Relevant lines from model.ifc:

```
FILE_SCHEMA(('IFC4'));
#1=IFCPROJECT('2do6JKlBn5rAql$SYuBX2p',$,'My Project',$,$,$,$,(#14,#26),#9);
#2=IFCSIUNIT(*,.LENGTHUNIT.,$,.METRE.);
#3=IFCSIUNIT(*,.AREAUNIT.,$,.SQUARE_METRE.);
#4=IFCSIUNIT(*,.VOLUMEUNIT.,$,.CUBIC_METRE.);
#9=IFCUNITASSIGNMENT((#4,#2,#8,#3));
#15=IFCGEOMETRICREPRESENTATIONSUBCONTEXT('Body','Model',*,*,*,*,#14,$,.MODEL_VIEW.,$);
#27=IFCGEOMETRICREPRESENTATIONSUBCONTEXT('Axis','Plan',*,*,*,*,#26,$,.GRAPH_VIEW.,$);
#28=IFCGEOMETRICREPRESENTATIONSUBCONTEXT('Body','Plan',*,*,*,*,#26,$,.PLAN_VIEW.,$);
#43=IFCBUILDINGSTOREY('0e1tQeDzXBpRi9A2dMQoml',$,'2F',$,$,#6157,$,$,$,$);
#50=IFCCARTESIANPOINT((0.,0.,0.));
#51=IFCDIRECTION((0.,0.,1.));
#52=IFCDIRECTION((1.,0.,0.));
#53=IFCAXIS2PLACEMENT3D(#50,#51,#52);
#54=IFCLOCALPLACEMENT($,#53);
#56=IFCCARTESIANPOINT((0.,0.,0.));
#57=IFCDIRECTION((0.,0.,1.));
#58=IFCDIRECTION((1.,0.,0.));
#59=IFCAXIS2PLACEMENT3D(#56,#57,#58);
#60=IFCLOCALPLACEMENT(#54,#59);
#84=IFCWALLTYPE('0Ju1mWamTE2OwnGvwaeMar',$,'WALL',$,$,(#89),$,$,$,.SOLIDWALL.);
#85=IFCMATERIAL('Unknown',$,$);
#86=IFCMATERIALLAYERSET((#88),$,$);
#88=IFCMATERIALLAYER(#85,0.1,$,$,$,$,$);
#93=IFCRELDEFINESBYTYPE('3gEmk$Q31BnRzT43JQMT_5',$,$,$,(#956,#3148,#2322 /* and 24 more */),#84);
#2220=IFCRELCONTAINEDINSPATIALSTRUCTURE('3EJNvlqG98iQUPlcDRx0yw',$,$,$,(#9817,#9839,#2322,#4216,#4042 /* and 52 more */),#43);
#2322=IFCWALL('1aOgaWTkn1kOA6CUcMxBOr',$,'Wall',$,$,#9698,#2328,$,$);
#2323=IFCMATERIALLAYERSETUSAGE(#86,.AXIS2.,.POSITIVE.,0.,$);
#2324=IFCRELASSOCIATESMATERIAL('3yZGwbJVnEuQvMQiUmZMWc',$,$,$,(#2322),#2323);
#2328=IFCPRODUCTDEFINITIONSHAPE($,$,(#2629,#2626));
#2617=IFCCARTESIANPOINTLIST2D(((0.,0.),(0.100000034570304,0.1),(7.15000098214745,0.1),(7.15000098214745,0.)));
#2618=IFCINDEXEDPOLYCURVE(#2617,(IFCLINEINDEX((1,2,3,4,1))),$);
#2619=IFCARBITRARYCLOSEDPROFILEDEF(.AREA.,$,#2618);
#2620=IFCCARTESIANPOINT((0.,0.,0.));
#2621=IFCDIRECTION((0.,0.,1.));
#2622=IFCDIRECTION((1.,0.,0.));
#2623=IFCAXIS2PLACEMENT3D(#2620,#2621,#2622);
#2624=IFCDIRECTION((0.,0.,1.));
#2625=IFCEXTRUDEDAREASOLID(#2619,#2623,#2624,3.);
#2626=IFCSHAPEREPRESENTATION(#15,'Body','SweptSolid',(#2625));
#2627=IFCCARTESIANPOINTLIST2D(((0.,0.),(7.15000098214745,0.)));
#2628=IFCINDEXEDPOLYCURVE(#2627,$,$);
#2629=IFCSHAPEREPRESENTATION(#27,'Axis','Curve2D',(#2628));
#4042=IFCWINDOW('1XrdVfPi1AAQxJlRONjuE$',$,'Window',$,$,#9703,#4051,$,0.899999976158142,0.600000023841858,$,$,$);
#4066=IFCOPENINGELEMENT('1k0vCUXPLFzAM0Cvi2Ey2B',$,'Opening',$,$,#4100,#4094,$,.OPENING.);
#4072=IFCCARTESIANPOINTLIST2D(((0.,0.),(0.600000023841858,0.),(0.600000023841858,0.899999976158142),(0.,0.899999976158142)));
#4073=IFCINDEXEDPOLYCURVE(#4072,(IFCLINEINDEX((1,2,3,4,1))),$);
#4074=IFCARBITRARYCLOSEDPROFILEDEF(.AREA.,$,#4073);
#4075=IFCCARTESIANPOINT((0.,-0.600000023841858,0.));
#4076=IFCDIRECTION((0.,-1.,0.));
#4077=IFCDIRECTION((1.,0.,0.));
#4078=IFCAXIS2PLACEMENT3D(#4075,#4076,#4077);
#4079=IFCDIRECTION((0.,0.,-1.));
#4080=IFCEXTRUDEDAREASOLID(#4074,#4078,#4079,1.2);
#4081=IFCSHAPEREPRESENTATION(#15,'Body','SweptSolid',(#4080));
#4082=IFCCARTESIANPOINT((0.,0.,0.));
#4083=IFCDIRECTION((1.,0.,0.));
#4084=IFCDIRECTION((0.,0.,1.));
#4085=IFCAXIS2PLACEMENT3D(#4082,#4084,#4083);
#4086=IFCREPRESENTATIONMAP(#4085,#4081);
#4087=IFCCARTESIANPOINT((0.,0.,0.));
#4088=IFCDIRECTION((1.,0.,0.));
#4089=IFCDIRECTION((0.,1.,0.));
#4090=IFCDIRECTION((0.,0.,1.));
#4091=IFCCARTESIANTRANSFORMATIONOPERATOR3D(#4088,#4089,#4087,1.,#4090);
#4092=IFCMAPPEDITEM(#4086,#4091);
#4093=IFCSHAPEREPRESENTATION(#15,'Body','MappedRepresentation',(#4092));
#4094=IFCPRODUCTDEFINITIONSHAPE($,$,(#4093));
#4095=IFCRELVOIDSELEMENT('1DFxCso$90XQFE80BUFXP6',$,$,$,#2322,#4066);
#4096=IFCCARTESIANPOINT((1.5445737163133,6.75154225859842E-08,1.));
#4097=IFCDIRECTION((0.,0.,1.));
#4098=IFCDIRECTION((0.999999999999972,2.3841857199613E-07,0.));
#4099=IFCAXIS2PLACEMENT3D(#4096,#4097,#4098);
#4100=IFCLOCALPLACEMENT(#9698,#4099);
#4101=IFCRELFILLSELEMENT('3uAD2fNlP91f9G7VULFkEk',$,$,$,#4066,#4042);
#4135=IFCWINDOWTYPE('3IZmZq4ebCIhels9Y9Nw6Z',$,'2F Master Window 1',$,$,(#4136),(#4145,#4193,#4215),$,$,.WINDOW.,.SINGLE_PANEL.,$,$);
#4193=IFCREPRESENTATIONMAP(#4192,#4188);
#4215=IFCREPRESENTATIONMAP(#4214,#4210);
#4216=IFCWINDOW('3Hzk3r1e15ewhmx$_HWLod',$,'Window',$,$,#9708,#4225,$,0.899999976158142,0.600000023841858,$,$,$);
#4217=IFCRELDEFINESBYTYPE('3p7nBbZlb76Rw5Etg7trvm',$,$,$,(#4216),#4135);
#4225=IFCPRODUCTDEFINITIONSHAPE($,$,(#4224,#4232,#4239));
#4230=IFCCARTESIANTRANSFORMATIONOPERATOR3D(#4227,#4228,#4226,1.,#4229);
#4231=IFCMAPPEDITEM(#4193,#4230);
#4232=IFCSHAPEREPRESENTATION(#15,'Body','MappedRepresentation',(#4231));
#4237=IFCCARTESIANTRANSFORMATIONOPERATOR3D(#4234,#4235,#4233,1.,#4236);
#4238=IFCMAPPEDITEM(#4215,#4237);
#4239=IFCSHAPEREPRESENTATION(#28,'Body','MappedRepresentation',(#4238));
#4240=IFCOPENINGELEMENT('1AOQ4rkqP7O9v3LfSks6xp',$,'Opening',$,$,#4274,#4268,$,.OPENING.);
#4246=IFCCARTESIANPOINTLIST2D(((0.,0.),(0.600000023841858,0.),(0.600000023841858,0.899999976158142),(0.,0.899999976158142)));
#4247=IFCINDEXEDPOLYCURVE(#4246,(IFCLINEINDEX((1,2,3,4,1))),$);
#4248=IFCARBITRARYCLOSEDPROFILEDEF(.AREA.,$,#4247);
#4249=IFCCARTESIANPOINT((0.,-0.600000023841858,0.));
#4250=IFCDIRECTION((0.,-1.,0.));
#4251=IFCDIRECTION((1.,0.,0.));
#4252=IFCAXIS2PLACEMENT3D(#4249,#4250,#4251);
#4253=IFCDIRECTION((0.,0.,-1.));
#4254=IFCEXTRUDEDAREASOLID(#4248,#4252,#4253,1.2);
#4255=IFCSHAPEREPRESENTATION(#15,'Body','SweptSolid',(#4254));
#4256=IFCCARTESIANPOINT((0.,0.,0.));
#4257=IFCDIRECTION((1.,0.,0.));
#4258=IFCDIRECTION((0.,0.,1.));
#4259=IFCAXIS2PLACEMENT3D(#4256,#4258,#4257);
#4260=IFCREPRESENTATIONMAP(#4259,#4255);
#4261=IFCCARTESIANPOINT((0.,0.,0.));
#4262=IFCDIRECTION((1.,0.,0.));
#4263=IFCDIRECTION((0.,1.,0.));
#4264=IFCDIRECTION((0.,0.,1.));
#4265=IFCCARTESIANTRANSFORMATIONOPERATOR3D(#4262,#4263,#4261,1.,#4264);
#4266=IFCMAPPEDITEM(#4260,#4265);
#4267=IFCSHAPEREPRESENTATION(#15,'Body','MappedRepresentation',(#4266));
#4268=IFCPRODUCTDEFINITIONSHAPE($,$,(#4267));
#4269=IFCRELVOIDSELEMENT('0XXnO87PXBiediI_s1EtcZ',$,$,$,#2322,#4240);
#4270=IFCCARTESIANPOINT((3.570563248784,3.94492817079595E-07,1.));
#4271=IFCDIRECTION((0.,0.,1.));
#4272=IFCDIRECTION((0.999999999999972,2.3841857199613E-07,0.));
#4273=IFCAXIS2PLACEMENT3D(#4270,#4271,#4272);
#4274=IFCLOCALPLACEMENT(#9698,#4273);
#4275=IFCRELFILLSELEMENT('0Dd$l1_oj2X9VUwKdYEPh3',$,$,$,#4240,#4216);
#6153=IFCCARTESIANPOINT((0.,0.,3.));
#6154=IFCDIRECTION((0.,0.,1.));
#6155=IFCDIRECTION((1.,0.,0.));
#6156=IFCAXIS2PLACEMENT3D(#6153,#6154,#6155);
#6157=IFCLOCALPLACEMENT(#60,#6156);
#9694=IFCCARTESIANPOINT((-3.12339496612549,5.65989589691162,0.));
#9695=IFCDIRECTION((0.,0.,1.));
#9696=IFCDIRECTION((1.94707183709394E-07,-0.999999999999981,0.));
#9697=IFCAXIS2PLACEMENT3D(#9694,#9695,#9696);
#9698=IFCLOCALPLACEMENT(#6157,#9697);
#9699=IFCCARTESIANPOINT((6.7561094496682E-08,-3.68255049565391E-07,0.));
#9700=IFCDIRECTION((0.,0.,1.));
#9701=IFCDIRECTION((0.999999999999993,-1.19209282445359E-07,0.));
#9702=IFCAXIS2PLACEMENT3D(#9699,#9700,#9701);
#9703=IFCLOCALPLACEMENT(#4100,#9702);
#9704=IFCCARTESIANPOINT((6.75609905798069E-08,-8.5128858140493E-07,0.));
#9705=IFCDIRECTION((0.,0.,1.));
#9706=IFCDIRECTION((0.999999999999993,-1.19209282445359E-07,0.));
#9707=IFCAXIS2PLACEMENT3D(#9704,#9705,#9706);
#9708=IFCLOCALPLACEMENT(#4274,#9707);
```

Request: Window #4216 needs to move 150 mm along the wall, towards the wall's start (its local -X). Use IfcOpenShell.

```python
import ifcopenshell
import ifcopenshell.api.geometry
import ifcopenshell.util.placement
import ifcopenshell.util.unit

model = ifcopenshell.open("model.ifc")
unit_scale = ifcopenshell.util.unit.calculate_unit_scale(model)

window = model.by_guid("3Hzk3r1e15ewhmx$_HWLod")
opening = window.FillsVoids[0].RelatingOpeningElement
wall = opening.VoidsElements[0].RelatingBuildingElement

wall_matrix = ifcopenshell.util.placement.get_local_placement(wall.ObjectPlacement)
shift = wall_matrix[:3, 0] * -0.15 / unit_scale
before = ifcopenshell.util.placement.get_local_placement(window.ObjectPlacement)[:3, 3].copy()

# The window is placed relative to its opening, so it follows when the opening moves.
matrix = ifcopenshell.util.placement.get_local_placement(opening.ObjectPlacement)
matrix[:3, 3] += shift
ifcopenshell.api.geometry.edit_object_placement(
    model, product=opening, matrix=matrix, is_si=False, should_transform_children=True
)

after = ifcopenshell.util.placement.get_local_placement(window.ObjectPlacement)[:3, 3]
print("window moved by", (after - before).round(3) + 0.0)

model.write("model_v2.ifc")
```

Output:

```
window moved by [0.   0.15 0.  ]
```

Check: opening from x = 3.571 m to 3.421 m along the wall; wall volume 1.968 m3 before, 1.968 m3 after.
